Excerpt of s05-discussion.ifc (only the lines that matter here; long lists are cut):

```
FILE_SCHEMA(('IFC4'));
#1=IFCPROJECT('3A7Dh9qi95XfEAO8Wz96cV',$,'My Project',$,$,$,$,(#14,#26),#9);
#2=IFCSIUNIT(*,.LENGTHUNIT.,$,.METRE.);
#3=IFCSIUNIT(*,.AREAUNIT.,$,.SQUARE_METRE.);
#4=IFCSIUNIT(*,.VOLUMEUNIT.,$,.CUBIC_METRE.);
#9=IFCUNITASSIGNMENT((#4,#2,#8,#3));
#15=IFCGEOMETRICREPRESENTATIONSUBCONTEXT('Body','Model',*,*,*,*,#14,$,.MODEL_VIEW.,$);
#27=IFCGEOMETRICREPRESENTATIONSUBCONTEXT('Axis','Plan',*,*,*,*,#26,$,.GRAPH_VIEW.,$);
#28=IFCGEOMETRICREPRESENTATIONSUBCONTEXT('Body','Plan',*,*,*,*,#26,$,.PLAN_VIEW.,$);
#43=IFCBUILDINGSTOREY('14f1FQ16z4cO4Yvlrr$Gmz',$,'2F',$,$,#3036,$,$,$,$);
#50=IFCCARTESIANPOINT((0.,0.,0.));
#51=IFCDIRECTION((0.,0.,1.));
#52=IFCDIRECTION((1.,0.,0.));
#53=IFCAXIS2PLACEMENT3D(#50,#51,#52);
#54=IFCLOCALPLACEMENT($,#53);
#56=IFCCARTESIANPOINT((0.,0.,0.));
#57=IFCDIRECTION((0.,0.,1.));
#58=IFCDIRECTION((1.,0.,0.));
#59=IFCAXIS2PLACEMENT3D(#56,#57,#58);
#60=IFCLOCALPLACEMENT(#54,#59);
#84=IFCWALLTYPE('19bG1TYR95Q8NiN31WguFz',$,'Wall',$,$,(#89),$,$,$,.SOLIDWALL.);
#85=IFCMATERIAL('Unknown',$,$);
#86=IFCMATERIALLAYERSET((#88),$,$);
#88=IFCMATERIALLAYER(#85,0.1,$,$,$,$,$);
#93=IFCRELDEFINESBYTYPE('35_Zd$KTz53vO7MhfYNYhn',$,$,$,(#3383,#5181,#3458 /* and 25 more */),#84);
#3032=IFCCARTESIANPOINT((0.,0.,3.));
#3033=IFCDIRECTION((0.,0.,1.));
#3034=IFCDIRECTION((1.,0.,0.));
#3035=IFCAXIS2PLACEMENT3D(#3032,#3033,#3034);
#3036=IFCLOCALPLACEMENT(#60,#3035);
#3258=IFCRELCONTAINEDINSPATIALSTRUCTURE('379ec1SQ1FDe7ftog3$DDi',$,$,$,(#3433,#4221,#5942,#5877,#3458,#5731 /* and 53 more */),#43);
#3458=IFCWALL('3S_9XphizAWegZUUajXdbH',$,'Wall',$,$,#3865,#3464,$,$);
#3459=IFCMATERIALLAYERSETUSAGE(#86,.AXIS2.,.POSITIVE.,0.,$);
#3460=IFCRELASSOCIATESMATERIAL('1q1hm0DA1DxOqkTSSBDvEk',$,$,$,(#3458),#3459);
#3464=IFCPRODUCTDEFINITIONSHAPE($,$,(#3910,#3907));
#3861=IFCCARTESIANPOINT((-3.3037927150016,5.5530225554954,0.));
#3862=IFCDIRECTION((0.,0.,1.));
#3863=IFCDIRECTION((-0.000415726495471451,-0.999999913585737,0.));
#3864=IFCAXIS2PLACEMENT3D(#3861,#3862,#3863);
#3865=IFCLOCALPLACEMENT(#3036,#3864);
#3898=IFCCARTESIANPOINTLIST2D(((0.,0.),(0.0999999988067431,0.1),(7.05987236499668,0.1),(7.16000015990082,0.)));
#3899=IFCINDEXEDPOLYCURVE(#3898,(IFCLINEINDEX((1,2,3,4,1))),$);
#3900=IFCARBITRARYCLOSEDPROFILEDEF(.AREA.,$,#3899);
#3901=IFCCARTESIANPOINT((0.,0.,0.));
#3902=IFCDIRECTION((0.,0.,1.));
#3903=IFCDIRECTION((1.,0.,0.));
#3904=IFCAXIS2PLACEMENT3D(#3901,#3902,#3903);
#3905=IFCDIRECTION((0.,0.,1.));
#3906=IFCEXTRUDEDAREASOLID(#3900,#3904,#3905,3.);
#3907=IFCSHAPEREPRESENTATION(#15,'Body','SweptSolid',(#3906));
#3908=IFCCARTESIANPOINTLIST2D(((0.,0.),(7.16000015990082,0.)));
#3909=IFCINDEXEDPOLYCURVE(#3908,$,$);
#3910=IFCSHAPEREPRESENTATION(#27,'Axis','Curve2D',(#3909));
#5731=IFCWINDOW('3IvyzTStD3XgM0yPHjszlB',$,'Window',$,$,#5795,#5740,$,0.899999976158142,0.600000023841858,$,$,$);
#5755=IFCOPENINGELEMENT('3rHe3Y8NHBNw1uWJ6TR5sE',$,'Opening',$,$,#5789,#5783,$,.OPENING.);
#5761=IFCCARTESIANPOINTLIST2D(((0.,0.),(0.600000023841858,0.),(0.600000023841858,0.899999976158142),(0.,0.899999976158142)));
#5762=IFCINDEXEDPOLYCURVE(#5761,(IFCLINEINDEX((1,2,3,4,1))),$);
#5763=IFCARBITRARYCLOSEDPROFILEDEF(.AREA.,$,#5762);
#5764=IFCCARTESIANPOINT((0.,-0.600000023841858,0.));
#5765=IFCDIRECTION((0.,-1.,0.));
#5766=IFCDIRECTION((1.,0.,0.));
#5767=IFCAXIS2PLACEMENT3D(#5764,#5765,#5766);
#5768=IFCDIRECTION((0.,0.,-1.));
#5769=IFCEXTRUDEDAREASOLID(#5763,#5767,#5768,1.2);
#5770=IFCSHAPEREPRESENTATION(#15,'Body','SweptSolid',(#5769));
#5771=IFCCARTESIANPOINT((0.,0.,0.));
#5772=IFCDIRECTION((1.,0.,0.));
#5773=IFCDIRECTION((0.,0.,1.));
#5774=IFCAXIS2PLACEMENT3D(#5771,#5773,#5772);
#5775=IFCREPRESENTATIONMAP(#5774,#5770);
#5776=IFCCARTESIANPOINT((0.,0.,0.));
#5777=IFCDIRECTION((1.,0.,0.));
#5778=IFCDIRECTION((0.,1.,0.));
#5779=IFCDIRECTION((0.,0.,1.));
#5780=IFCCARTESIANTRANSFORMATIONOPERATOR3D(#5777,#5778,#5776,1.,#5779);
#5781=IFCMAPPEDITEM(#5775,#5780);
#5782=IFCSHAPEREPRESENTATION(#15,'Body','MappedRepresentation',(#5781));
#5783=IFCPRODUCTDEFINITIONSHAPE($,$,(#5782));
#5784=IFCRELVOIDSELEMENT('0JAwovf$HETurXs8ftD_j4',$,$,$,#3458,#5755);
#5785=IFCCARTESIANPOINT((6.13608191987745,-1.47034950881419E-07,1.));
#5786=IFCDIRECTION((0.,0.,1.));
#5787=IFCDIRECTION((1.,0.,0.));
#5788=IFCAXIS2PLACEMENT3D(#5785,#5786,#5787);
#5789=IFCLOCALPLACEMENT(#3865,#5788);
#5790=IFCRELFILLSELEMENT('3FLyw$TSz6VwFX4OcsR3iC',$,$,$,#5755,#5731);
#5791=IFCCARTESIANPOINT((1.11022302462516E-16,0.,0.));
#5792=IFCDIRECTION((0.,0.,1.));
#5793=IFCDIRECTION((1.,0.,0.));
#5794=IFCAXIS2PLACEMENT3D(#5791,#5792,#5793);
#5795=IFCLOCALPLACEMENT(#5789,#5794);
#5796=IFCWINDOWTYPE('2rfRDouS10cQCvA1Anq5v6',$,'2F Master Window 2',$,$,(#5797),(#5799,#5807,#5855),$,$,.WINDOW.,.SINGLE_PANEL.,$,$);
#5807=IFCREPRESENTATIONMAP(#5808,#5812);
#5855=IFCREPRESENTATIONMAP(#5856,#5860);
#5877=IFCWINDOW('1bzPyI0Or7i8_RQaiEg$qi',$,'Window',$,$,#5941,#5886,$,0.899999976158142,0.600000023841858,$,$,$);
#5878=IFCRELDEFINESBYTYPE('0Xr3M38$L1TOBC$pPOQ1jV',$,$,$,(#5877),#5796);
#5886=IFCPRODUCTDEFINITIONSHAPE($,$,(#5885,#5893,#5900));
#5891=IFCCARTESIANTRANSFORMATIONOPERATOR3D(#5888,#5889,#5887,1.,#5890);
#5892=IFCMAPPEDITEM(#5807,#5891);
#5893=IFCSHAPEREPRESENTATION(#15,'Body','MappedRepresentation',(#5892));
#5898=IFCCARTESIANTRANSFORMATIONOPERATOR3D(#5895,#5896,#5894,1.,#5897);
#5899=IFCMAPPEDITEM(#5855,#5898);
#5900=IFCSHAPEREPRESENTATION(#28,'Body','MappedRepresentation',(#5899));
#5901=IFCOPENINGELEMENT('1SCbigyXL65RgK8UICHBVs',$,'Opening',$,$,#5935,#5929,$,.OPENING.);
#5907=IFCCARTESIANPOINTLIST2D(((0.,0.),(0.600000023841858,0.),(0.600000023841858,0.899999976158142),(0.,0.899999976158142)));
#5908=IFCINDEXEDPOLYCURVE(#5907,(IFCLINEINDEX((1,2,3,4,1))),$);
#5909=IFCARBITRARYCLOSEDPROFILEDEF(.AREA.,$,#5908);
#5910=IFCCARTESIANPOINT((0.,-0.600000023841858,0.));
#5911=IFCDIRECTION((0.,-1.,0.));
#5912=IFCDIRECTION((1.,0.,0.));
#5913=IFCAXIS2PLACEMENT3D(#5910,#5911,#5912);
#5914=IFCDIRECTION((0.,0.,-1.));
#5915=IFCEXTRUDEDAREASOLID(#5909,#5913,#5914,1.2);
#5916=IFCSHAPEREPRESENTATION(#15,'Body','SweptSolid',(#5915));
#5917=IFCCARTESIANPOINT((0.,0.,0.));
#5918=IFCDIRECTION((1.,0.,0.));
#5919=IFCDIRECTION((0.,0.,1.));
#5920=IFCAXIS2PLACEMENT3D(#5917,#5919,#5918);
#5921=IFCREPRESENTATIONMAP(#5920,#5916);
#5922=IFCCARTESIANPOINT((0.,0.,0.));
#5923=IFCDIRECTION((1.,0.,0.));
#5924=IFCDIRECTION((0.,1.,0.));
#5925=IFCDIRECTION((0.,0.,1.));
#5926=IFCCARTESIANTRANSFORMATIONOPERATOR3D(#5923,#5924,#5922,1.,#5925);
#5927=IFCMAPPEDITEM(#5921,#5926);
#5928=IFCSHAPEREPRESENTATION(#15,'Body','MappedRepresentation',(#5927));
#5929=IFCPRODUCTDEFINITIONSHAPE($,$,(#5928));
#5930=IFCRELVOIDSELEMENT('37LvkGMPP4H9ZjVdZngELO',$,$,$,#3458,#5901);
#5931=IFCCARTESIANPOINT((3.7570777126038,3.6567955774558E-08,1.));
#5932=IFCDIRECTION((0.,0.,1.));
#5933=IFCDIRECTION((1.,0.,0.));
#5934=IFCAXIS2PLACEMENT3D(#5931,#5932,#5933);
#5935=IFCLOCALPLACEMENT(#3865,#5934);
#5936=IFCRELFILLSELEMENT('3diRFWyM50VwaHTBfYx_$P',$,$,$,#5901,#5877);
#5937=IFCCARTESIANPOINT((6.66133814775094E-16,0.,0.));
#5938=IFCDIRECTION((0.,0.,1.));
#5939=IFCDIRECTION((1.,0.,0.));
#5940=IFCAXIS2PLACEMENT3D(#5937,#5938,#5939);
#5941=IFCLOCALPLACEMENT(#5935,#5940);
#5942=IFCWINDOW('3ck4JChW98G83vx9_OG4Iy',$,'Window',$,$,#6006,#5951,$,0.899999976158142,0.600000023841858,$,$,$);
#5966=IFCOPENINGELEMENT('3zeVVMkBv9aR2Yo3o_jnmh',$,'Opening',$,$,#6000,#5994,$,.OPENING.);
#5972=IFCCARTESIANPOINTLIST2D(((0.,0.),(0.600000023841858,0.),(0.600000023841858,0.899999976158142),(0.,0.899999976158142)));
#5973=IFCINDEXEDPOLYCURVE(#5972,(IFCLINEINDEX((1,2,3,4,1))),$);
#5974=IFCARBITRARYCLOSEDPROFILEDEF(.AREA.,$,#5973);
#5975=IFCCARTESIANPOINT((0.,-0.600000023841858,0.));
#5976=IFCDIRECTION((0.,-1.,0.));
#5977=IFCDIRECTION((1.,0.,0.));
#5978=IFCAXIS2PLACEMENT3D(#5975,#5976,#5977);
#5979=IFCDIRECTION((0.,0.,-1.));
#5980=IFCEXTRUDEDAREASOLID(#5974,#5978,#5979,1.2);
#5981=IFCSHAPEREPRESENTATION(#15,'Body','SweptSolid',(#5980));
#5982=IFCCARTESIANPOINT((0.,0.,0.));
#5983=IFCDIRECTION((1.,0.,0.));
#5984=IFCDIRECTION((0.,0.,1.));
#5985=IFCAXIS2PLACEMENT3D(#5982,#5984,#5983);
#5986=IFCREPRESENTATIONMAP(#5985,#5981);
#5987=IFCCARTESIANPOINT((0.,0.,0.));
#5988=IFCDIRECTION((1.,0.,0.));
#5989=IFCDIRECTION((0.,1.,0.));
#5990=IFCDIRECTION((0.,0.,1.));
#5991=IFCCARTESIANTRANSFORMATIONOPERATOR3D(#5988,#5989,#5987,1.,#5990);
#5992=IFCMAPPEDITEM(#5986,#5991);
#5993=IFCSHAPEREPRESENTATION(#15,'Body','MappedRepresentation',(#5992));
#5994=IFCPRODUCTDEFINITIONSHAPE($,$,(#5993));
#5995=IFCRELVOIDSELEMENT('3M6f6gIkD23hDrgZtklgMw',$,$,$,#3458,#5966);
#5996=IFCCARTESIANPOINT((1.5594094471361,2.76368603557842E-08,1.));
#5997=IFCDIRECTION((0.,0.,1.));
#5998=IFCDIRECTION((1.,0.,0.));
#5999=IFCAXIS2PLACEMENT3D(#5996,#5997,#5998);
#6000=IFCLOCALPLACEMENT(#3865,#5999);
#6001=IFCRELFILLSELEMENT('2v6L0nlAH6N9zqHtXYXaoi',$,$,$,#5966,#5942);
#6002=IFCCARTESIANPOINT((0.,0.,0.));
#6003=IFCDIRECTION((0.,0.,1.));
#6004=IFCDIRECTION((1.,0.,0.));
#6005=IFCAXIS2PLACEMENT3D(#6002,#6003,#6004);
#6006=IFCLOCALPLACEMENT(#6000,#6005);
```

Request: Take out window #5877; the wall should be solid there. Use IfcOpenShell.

```python
import ifcopenshell
import ifcopenshell.api.feature
import ifcopenshell.api.root
import ifcopenshell.geom
import ifcopenshell.util.shape

model = ifcopenshell.open("s05-discussion.ifc")
settings = ifcopenshell.geom.settings()


def volume(element):
    """Net volume in cubic metres, openings subtracted."""
    shape = ifcopenshell.geom.create_shape(settings, element)
    return ifcopenshell.util.shape.get_volume(shape.geometry)


window = model.by_id(5877)
opening = window.FillsVoids[0].RelatingOpeningElement
wall = opening.VoidsElements[0].RelatingBuildingElement
before = volume(wall)

ifcopenshell.api.root.remove_product(model, product=window)
ifcopenshell.api.feature.remove_feature(model, feature=opening)

after = volume(wall)

print(f"wall volume {before:.3f} -> {after:.3f} m3")

model.write("s05-discussion_v2.ifc")
```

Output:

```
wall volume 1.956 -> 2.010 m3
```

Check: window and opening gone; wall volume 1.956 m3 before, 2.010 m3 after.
